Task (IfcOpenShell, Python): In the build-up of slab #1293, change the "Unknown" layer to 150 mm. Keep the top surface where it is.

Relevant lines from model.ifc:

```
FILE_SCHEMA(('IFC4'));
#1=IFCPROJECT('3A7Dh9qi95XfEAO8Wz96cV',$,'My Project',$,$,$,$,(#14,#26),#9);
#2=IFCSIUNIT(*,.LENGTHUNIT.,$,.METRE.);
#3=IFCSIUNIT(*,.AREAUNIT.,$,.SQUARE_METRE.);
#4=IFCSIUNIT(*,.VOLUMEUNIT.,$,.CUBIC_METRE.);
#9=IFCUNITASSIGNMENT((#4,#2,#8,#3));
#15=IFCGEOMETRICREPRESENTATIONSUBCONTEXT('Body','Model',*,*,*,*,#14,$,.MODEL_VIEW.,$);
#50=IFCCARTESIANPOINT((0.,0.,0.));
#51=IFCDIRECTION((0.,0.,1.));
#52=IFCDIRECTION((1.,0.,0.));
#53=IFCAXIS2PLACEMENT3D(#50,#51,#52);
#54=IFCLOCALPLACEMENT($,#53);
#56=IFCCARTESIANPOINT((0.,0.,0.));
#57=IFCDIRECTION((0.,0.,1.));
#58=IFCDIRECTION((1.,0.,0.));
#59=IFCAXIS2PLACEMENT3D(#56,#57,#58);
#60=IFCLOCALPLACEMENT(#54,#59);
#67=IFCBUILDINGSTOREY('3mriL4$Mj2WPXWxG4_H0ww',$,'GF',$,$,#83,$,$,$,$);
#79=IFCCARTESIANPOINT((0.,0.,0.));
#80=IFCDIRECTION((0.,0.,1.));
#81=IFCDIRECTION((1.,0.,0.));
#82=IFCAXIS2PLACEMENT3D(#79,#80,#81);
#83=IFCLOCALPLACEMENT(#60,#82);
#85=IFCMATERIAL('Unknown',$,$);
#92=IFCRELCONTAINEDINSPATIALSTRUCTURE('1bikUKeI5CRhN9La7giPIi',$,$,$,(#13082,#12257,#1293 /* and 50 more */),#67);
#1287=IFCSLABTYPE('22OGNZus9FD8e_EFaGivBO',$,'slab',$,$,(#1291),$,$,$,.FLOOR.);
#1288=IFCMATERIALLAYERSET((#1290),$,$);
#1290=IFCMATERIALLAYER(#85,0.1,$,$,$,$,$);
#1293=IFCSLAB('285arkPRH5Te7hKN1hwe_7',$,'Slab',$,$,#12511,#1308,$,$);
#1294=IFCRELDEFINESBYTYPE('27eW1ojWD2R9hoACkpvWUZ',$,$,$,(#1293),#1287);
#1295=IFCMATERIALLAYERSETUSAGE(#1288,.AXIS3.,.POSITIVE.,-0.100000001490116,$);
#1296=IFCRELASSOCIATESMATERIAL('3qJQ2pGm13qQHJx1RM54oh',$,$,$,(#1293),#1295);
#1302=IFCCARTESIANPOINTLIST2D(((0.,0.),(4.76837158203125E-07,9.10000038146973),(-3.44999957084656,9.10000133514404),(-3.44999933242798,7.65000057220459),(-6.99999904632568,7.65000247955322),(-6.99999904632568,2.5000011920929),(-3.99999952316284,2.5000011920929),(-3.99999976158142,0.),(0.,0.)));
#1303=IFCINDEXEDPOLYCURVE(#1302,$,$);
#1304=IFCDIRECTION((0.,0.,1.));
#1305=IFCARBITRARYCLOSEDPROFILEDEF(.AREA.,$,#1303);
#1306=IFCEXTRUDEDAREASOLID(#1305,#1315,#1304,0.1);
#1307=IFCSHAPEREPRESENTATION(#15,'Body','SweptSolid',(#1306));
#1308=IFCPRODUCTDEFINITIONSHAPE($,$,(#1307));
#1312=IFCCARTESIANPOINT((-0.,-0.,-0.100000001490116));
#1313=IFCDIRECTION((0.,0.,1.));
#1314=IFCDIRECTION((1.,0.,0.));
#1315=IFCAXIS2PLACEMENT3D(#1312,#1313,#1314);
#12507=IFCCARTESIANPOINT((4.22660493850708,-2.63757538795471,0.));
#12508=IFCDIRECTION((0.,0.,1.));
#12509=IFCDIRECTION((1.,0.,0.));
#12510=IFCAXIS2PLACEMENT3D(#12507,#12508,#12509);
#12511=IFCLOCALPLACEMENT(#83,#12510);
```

```python
import ifcopenshell
import ifcopenshell.util.element
import ifcopenshell.util.representation
import ifcopenshell.util.unit

model = ifcopenshell.open("model.ifc")
unit_scale = ifcopenshell.util.unit.calculate_unit_scale(model)

layer_set = model.by_id(1288)
layer = next(l for l in layer_set.MaterialLayers if l.Material and l.Material.Name == "Unknown")
change = 0.15 / unit_scale - layer.LayerThickness
layer.LayerThickness += change

# Geometry does not follow the layer set by itself.
slabs = [e for e in ifcopenshell.util.element.get_elements_by_material(model, layer_set) if e.is_a("IfcSlab")]
for slab in sorted(slabs, key=lambda e: e.id()):
    body = ifcopenshell.util.representation.get_representation(slab, "Model", "Body")
    solid = body.Items[0]
    old_depth = solid.Depth
    solid.Depth += change
    # Extruded upwards: lower the start of the extrusion so the top stays.
    x, y, z = solid.Position.Location.Coordinates
    solid.Position.Location = model.createIfcCartesianPoint((x, y, z - change))
    print(slab.id(), f"{old_depth:g} -> {solid.Depth:g}")

# The layers are counted up from the underside, which has moved.
for usage in {ifcopenshell.util.element.get_material(slab) for slab in slabs}:
    usage.OffsetFromReferenceLine -= change

model.write("model_v2.ifc")
```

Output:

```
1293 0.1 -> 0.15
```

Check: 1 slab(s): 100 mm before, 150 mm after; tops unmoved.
